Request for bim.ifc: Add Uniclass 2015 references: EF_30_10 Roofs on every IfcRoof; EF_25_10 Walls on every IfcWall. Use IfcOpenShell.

First a look at what the model holds.

```python
import ifcopenshell

model = ifcopenshell.open("bim.ifc")
print(model.schema)
print("classifications:", [c.Name for c in model.by_type("IfcClassification")])
for ifc_class in ("IfcDoor", "IfcRoof", "IfcStair", "IfcWall", "IfcWindow"):
    print(ifc_class, len(model.by_type(ifc_class)))
```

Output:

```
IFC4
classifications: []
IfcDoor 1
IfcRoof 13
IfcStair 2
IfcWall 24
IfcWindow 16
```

```python
import ifcopenshell
import ifcopenshell.api.classification

model = ifcopenshell.open("bim.ifc")

system = ifcopenshell.api.classification.add_classification(model, classification="Uniclass 2015")

codes = {
    "IfcRoof": ("EF_30_10", "Roofs"),
    "IfcWall": ("EF_25_10", "Walls"),
}
for ifc_class, (code, name) in codes.items():
    products = model.by_type(ifc_class)
    ifcopenshell.api.classification.add_reference(
        model, products=products, classification=system, identification=code, name=name
    )
    print(code, len(products))

model.write("bim_v2.ifc")
```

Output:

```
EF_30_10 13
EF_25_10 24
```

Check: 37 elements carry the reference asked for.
